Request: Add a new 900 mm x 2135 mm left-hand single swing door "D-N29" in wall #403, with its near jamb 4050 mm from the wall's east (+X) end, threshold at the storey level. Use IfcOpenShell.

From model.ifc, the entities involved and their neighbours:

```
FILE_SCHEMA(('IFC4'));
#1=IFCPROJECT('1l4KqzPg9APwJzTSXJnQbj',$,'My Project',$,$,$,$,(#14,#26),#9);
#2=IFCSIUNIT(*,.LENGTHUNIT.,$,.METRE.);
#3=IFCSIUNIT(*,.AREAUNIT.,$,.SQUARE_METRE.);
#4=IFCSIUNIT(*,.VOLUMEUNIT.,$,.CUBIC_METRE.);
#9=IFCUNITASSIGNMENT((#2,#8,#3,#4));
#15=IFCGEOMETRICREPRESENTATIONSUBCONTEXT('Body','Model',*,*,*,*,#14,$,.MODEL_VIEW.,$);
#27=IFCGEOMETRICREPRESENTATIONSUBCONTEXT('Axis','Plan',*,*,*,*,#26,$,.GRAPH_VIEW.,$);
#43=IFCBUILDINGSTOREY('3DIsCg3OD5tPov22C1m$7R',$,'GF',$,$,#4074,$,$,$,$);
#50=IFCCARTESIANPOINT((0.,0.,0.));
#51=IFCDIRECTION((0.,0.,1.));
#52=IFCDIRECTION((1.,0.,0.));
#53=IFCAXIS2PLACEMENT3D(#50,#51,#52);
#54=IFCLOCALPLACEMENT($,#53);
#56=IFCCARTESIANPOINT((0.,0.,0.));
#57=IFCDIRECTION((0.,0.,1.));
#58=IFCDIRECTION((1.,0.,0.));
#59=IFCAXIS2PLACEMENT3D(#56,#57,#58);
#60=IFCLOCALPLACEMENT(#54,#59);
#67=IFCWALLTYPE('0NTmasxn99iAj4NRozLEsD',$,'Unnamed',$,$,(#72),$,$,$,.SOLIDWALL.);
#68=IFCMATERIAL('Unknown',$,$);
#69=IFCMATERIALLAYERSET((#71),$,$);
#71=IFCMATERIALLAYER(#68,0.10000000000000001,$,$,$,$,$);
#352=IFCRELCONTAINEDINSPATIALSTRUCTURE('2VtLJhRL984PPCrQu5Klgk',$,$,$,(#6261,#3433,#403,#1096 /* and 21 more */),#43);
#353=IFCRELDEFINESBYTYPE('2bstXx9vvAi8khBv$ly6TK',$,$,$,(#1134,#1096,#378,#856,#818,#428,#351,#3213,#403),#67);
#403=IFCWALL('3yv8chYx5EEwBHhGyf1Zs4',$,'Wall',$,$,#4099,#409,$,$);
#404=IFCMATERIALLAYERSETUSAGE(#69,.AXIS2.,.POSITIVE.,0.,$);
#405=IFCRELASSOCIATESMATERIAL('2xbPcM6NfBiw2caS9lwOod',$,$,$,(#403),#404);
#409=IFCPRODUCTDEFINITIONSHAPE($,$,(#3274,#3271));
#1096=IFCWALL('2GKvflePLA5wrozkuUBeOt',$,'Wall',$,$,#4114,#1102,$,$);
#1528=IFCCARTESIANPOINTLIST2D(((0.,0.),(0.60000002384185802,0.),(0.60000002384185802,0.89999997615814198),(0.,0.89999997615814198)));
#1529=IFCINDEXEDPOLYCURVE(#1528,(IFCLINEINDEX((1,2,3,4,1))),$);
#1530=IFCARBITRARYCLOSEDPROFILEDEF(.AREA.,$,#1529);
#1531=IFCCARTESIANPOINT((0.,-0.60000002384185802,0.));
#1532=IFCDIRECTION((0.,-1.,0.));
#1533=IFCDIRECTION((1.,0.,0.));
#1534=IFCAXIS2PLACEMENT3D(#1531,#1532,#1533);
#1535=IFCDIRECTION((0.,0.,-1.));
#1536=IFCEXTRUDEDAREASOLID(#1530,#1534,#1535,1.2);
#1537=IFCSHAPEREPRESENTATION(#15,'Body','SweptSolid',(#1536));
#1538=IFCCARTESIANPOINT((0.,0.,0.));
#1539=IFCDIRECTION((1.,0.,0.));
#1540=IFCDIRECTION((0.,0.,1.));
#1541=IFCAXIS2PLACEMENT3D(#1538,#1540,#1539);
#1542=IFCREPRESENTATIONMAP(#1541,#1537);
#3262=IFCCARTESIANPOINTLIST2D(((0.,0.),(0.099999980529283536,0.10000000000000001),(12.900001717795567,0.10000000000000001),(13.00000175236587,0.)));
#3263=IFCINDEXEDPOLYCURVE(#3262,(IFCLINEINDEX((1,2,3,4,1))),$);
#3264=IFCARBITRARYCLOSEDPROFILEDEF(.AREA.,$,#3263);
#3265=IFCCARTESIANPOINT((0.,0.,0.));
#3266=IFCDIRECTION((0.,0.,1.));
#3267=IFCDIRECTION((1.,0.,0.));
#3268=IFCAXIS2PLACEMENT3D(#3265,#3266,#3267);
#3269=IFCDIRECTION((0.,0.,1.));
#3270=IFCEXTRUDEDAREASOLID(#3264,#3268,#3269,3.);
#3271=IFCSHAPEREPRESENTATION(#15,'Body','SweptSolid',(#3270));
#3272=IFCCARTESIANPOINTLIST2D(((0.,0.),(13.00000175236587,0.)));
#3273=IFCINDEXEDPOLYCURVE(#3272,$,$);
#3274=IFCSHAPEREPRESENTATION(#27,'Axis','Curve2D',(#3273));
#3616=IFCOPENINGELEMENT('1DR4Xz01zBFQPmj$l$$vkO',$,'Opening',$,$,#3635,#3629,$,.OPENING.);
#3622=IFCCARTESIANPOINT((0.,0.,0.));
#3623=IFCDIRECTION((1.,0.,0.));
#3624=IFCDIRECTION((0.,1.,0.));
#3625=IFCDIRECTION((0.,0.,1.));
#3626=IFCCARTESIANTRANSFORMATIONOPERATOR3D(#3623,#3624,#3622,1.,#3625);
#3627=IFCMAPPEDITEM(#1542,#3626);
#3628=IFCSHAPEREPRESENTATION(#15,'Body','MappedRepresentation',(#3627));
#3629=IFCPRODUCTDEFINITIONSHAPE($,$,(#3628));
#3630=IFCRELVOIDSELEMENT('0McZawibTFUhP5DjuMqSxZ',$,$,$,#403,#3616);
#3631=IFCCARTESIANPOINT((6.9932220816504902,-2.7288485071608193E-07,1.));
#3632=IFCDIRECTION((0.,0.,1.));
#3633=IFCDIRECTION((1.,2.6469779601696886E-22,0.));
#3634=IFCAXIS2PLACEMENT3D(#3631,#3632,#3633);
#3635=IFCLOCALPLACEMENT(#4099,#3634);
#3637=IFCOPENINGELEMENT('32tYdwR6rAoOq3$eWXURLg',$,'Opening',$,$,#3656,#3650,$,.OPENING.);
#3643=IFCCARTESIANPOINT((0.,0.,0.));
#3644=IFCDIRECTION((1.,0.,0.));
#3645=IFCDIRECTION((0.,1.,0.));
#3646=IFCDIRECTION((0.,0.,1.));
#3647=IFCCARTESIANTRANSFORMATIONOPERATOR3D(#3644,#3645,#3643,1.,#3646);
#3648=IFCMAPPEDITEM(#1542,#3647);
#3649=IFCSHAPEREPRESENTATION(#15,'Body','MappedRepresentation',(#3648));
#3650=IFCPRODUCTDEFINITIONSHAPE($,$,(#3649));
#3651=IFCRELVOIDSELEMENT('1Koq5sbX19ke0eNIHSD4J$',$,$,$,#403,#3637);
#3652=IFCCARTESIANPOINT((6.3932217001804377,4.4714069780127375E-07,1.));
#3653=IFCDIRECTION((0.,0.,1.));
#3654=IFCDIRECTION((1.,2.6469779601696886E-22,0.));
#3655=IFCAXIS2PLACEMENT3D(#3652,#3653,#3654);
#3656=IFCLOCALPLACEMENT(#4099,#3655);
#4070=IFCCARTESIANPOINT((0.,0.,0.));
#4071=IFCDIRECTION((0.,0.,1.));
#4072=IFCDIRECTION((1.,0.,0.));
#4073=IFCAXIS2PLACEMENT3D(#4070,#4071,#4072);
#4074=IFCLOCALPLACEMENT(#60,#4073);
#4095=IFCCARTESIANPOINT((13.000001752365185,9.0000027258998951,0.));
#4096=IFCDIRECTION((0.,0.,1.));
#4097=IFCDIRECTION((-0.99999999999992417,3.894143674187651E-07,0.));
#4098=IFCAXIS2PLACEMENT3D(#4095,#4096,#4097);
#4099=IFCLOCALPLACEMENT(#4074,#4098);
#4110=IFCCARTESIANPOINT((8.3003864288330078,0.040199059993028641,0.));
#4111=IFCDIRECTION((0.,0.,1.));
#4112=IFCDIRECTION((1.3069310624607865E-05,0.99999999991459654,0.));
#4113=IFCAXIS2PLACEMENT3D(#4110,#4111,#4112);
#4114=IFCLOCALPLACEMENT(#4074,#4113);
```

```python
import numpy as np
import ifcopenshell
import ifcopenshell.api.feature
import ifcopenshell.api.geometry
import ifcopenshell.api.root
import ifcopenshell.api.spatial
import ifcopenshell.geom
import ifcopenshell.util.element
import ifcopenshell.util.placement
import ifcopenshell.util.representation
import ifcopenshell.util.shape
import ifcopenshell.util.unit

model = ifcopenshell.open("model.ifc")
unit_scale = ifcopenshell.util.unit.calculate_unit_scale(model)
settings = ifcopenshell.geom.settings()


def volume(element):
    """Net volume in cubic metres, openings subtracted."""
    shape = ifcopenshell.geom.create_shape(settings, element)
    return ifcopenshell.util.shape.get_volume(shape.geometry)


wall = model.by_id(403)
storey = ifcopenshell.util.element.get_container(wall, ifc_class="IfcBuildingStorey")
context = ifcopenshell.util.representation.get_context(model, "Model", "Body", "MODEL_VIEW")
before = volume(wall)

width, height, from_end, sill = 0.9, 2.135, 4.05, 0.0  # metres

# The wall runs along its own X axis, and the end named is its -X end.
wall_shape = ifcopenshell.geom.create_shape(settings, wall)
x, y, z = ifcopenshell.util.shape.get_vertices(wall_shape.geometry).T
start = x.min() + from_end
face, thickness = float(y.min()), float(y.max() - y.min())
wall_matrix = ifcopenshell.util.placement.get_local_placement(wall.ObjectPlacement)
level = ifcopenshell.util.placement.get_local_placement(storey.ObjectPlacement)[2, 3]


def in_wall(x, y):
    """Placement at x, y metres in the wall's axes, at sill height."""
    matrix = wall_matrix.copy()
    matrix[:, 3] = wall_matrix @ np.array([x / unit_scale, y / unit_scale, 0.0, 1.0])
    matrix[2, 3] = level + sill / unit_scale
    return matrix


# Opening: a box that overshoots both wall faces by 50 mm.
opening = ifcopenshell.api.root.create_entity(model, ifc_class="IfcOpeningElement", predefined_type="OPENING")
box = ifcopenshell.api.geometry.add_wall_representation(
    model, context=context, length=width, height=height, thickness=thickness + 0.1
)
ifcopenshell.api.geometry.assign_representation(model, product=opening, representation=box)
ifcopenshell.api.geometry.edit_object_placement(model, product=opening, matrix=in_wall(start, face - 0.05), is_si=False)
ifcopenshell.api.feature.add_feature(model, feature=opening, element=wall)

door = ifcopenshell.api.root.create_entity(model, ifc_class="IfcDoor", name="D-N29", predefined_type="DOOR")
door.OverallWidth, door.OverallHeight = width / unit_scale, height / unit_scale
door.OperationType = "SINGLE_SWING_LEFT"
body = ifcopenshell.api.geometry.add_door_representation(
    model,
    context=context,
    overall_width=door.OverallWidth,
    overall_height=door.OverallHeight,
    operation_type="SINGLE_SWING_LEFT",
    lining_properties={"LiningDepth": thickness / unit_scale, "ThresholdDepth": thickness / unit_scale},
)
ifcopenshell.api.geometry.assign_representation(model, product=door, representation=body)
ifcopenshell.api.spatial.assign_container(model, products=[door], relating_structure=storey)
ifcopenshell.api.feature.add_filling(model, opening=opening, element=door)

# The lining spans the wall, so the door starts at the wall face.
ifcopenshell.api.geometry.edit_object_placement(model, product=door, matrix=in_wall(start, face), is_si=False)

after = volume(wall)

print(f"wall volume {before:.3f} -> {after:.3f} m3")

model.write("model_v2.ifc")
```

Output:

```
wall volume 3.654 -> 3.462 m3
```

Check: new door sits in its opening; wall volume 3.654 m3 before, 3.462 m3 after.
